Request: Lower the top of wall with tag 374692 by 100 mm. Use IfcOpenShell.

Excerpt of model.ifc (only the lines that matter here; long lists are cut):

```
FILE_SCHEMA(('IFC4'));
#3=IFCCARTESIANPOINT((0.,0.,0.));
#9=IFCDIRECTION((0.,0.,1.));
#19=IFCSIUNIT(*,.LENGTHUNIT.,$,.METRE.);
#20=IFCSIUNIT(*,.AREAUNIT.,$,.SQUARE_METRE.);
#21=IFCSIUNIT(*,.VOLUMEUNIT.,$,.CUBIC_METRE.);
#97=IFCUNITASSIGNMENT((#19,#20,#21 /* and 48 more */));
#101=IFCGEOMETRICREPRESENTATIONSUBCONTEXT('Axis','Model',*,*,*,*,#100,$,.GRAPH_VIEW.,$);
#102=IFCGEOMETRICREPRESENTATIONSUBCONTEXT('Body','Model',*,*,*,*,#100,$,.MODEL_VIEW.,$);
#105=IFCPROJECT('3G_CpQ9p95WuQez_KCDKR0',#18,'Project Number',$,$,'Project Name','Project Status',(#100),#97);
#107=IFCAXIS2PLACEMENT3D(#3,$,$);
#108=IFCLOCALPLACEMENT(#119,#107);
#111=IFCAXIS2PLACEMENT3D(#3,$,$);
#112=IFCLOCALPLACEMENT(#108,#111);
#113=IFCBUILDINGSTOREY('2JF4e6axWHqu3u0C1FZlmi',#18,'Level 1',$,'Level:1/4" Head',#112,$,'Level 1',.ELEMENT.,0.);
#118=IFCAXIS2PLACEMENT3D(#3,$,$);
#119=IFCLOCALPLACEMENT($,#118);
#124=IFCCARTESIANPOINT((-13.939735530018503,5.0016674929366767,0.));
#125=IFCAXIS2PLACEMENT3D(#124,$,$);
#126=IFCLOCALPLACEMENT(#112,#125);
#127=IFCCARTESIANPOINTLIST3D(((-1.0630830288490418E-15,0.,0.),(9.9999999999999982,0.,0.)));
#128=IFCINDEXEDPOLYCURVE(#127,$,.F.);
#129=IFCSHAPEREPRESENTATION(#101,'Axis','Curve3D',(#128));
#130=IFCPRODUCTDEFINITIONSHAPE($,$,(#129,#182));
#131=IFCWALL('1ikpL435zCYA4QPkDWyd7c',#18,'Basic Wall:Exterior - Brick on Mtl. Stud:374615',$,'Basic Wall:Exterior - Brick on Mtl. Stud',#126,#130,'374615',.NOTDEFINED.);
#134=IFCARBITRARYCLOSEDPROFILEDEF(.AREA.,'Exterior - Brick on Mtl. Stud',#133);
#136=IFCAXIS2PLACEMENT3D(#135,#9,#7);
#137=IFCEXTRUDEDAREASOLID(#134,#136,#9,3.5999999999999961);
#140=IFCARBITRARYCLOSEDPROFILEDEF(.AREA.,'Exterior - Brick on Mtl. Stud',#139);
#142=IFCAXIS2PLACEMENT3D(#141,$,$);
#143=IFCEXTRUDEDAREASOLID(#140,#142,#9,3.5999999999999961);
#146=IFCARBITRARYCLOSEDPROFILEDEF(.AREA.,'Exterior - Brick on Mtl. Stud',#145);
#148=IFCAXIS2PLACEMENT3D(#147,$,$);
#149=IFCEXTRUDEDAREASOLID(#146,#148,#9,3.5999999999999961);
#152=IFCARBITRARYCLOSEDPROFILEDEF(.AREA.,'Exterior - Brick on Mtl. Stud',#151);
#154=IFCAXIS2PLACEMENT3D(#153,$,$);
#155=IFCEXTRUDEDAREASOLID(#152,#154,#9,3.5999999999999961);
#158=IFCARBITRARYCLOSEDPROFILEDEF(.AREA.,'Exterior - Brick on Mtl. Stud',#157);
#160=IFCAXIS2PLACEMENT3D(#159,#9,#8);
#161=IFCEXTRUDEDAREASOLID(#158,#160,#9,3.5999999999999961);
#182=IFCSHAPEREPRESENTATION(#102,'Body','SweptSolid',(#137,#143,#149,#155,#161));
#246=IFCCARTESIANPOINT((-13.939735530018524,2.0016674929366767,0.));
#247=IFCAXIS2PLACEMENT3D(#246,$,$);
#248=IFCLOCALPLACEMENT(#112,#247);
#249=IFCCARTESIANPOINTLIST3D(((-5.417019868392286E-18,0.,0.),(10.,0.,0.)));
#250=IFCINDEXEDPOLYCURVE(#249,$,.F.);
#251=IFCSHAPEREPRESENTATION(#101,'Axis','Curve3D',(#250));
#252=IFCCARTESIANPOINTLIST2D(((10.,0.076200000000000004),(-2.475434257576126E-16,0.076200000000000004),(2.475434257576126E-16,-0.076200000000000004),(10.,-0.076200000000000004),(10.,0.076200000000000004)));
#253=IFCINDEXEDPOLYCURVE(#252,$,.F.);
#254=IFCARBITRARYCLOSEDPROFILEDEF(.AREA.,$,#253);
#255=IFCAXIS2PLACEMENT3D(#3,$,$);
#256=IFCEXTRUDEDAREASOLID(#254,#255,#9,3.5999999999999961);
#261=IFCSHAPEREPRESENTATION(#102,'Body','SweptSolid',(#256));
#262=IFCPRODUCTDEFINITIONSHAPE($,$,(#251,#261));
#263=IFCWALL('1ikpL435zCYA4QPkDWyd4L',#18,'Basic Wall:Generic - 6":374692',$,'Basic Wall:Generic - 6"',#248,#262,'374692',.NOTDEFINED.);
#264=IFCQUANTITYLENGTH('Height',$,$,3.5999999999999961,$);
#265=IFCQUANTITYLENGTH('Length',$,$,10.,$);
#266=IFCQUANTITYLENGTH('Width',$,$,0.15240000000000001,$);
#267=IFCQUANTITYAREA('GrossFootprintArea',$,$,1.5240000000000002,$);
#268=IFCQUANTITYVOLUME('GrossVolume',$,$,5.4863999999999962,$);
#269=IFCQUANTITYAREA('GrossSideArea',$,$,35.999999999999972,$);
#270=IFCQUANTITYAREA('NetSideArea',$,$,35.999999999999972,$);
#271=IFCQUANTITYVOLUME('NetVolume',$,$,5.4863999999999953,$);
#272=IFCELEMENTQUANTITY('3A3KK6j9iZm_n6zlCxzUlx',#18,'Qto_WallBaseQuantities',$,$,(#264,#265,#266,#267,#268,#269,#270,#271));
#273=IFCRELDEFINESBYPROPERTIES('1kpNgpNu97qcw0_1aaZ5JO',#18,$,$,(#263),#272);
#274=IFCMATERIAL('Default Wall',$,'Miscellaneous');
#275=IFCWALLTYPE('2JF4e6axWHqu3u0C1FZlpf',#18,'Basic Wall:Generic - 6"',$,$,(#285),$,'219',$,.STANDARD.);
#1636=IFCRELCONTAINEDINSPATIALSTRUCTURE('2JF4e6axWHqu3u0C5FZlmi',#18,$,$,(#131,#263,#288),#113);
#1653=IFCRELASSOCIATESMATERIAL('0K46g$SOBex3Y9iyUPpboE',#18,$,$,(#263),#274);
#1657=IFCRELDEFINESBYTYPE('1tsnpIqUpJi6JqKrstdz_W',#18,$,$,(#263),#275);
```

```python
import ifcopenshell
import ifcopenshell.api.pset
import ifcopenshell.geom
import ifcopenshell.util.element
import ifcopenshell.util.representation
import ifcopenshell.util.shape
import ifcopenshell.util.unit

model = ifcopenshell.open("model.ifc")
unit_scale = ifcopenshell.util.unit.calculate_unit_scale(model)
area_scale = ifcopenshell.util.unit.calculate_unit_scale(model, "AREAUNIT")
volume_scale = ifcopenshell.util.unit.calculate_unit_scale(model, "VOLUMEUNIT")
settings = ifcopenshell.geom.settings()


def volume(element):
    """Net volume in cubic metres, openings subtracted."""
    shape = ifcopenshell.geom.create_shape(settings, element)
    return ifcopenshell.util.shape.get_volume(shape.geometry)


wall = model.by_id(263)
before = volume(wall)

body = ifcopenshell.util.representation.get_representation(wall, "Model", "Body")
solid = body.Items[0]
old_height = solid.Depth
solid.Depth -= 0.1 / unit_scale
after = volume(wall)
thickness = 0.1524  # wall thickness in metres

# Update the stored height, areas and volumes.
qto = model.by_id(ifcopenshell.util.element.get_pset(wall, "Qto_WallBaseQuantities", should_inherit=False)["id"])
ifcopenshell.api.pset.edit_qto(model, qto=qto, properties={
    "Height": solid.Depth,
    "GrossVolume": ifcopenshell.util.element.get_pset(wall, "Qto_WallBaseQuantities", "GrossVolume") * solid.Depth / old_height,
    "GrossSideArea": ifcopenshell.util.element.get_pset(wall, "Qto_WallBaseQuantities", "GrossSideArea") * solid.Depth / old_height,
    "NetSideArea": after / thickness / area_scale,
    "NetVolume": after / volume_scale,
})

print(f"height {old_height:g} -> {solid.Depth:g}, volume {before:.3f} -> {after:.3f} m3")

model.write("model_updated.ifc")
```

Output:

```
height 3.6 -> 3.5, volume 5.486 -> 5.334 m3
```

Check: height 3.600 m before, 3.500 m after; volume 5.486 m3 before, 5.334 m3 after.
